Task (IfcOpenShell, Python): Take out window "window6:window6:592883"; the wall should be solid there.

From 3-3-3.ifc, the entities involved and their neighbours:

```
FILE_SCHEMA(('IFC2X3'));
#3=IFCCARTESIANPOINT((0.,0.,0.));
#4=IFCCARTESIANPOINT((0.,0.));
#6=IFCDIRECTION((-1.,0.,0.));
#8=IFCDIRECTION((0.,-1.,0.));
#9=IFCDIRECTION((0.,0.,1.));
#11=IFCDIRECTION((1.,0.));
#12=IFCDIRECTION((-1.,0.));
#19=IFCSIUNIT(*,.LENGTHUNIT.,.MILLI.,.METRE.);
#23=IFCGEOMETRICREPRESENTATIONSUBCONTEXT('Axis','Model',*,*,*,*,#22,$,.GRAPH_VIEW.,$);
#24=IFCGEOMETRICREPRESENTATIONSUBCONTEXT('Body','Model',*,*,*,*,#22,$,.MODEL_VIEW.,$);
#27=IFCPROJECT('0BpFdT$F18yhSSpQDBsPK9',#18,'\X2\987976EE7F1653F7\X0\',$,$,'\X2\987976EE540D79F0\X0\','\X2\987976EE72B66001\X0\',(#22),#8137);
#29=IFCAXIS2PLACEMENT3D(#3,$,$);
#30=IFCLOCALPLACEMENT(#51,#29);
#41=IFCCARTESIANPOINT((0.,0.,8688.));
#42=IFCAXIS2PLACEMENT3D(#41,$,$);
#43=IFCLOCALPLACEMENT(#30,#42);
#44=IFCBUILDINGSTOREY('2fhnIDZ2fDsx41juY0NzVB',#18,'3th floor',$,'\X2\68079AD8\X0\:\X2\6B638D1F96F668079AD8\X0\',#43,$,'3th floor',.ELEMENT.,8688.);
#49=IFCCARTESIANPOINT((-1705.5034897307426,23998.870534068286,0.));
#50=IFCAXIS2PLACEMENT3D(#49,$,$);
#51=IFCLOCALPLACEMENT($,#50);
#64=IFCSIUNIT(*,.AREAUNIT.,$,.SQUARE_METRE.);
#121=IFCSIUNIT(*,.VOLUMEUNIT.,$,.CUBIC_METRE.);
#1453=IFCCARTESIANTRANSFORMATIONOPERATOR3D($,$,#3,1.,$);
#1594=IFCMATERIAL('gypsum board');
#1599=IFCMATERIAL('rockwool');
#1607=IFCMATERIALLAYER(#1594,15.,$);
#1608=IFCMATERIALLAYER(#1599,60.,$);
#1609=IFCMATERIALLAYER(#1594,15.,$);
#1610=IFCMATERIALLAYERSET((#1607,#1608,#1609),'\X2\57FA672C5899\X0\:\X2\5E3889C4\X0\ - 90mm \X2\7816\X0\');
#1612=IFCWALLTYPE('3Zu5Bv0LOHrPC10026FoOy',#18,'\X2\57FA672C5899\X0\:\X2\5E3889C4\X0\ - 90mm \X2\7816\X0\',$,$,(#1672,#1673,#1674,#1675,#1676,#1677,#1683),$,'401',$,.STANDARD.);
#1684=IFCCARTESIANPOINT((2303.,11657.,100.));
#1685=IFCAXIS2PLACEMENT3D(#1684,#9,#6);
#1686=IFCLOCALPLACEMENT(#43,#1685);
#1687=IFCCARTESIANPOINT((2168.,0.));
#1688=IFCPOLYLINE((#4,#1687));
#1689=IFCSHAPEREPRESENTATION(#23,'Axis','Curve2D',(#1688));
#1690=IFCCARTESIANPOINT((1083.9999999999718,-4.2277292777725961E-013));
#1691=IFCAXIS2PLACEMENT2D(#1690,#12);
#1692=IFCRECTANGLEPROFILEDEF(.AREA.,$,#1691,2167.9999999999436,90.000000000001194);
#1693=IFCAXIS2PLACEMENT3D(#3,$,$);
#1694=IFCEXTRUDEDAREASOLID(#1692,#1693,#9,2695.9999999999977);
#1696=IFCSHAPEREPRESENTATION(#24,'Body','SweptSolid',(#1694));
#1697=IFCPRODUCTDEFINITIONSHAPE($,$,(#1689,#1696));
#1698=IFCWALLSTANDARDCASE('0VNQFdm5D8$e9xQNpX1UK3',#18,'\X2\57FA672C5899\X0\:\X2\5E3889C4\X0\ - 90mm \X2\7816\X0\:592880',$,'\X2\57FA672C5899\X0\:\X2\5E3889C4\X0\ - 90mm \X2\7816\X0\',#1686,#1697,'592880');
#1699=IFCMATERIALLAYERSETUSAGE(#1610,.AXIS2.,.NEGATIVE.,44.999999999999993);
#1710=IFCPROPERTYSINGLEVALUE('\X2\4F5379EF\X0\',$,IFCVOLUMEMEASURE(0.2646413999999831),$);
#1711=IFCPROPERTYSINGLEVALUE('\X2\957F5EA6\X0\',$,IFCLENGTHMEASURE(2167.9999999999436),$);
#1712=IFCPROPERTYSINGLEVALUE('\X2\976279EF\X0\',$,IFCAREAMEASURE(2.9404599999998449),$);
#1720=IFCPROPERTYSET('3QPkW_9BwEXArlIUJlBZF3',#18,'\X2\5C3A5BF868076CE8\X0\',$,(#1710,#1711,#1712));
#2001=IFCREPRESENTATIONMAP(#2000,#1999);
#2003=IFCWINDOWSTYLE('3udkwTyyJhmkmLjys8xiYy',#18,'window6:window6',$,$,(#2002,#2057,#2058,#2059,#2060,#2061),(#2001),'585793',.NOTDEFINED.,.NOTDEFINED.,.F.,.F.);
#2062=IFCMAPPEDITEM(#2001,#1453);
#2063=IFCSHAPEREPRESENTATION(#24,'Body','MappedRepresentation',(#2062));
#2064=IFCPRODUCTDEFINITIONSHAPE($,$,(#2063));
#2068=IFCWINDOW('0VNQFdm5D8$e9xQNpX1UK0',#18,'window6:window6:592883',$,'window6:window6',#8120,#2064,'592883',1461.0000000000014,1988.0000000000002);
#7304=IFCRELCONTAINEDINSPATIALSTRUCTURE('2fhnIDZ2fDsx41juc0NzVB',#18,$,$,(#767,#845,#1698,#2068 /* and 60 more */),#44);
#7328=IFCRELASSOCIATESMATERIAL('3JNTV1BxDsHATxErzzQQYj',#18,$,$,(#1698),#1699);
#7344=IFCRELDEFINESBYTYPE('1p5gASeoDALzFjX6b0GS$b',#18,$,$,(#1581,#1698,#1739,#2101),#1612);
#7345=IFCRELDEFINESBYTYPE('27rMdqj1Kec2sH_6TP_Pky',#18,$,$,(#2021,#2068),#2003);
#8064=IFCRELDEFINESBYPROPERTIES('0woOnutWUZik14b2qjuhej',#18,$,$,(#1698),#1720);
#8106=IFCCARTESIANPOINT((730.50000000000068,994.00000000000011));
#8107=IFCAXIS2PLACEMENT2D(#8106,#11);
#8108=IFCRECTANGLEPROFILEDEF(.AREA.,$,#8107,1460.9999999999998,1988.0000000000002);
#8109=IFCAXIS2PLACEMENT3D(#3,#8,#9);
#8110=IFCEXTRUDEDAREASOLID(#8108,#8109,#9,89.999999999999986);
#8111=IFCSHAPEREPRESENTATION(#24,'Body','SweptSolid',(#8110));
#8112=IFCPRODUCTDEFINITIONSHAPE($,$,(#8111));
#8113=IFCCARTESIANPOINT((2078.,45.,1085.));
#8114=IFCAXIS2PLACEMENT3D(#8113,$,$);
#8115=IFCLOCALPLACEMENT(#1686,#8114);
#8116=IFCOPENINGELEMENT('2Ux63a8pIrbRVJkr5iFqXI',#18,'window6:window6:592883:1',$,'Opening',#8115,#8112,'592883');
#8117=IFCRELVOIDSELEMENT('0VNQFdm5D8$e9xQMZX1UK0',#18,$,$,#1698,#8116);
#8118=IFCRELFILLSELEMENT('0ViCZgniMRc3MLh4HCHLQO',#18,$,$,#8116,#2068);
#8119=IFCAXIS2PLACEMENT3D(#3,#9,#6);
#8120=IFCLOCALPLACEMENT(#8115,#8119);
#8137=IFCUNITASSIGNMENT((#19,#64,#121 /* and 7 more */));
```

```python
import ifcopenshell
import ifcopenshell.api.feature
import ifcopenshell.api.pset
import ifcopenshell.api.root
import ifcopenshell.geom
import ifcopenshell.util.element
import ifcopenshell.util.shape
import ifcopenshell.util.unit

model = ifcopenshell.open("3-3-3.ifc")
area_scale = ifcopenshell.util.unit.calculate_unit_scale(model, "AREAUNIT")
volume_scale = ifcopenshell.util.unit.calculate_unit_scale(model, "VOLUMEUNIT")
settings = ifcopenshell.geom.settings()


def volume(element):
    """Net volume in cubic metres, openings subtracted."""
    shape = ifcopenshell.geom.create_shape(settings, element)
    return ifcopenshell.util.shape.get_volume(shape.geometry)


window = model.by_guid("0VNQFdm5D8$e9xQNpX1UK0")
opening = window.FillsVoids[0].RelatingOpeningElement
wall = opening.VoidsElements[0].RelatingBuildingElement
before = volume(wall)

ifcopenshell.api.root.remove_product(model, product=window)
ifcopenshell.api.feature.remove_feature(model, feature=opening)

after = volume(wall)
thickness = 0.09  # wall thickness in metres

# Update the wall's stored quantities.
pset = model.by_id(ifcopenshell.util.element.get_pset(wall, "尺寸标注", should_inherit=False)["id"])
ifcopenshell.api.pset.edit_pset(model, pset=pset, properties={
    "体积": model.create_entity("IfcVolumeMeasure", after / volume_scale),
    "面积": model.create_entity("IfcAreaMeasure", after / thickness / area_scale),
})

print(f"wall volume {before:.3f} -> {after:.3f} m3")

model.write("3-3-3_rev.ifc")
```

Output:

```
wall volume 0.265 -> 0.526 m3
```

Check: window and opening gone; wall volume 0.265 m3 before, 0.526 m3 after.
